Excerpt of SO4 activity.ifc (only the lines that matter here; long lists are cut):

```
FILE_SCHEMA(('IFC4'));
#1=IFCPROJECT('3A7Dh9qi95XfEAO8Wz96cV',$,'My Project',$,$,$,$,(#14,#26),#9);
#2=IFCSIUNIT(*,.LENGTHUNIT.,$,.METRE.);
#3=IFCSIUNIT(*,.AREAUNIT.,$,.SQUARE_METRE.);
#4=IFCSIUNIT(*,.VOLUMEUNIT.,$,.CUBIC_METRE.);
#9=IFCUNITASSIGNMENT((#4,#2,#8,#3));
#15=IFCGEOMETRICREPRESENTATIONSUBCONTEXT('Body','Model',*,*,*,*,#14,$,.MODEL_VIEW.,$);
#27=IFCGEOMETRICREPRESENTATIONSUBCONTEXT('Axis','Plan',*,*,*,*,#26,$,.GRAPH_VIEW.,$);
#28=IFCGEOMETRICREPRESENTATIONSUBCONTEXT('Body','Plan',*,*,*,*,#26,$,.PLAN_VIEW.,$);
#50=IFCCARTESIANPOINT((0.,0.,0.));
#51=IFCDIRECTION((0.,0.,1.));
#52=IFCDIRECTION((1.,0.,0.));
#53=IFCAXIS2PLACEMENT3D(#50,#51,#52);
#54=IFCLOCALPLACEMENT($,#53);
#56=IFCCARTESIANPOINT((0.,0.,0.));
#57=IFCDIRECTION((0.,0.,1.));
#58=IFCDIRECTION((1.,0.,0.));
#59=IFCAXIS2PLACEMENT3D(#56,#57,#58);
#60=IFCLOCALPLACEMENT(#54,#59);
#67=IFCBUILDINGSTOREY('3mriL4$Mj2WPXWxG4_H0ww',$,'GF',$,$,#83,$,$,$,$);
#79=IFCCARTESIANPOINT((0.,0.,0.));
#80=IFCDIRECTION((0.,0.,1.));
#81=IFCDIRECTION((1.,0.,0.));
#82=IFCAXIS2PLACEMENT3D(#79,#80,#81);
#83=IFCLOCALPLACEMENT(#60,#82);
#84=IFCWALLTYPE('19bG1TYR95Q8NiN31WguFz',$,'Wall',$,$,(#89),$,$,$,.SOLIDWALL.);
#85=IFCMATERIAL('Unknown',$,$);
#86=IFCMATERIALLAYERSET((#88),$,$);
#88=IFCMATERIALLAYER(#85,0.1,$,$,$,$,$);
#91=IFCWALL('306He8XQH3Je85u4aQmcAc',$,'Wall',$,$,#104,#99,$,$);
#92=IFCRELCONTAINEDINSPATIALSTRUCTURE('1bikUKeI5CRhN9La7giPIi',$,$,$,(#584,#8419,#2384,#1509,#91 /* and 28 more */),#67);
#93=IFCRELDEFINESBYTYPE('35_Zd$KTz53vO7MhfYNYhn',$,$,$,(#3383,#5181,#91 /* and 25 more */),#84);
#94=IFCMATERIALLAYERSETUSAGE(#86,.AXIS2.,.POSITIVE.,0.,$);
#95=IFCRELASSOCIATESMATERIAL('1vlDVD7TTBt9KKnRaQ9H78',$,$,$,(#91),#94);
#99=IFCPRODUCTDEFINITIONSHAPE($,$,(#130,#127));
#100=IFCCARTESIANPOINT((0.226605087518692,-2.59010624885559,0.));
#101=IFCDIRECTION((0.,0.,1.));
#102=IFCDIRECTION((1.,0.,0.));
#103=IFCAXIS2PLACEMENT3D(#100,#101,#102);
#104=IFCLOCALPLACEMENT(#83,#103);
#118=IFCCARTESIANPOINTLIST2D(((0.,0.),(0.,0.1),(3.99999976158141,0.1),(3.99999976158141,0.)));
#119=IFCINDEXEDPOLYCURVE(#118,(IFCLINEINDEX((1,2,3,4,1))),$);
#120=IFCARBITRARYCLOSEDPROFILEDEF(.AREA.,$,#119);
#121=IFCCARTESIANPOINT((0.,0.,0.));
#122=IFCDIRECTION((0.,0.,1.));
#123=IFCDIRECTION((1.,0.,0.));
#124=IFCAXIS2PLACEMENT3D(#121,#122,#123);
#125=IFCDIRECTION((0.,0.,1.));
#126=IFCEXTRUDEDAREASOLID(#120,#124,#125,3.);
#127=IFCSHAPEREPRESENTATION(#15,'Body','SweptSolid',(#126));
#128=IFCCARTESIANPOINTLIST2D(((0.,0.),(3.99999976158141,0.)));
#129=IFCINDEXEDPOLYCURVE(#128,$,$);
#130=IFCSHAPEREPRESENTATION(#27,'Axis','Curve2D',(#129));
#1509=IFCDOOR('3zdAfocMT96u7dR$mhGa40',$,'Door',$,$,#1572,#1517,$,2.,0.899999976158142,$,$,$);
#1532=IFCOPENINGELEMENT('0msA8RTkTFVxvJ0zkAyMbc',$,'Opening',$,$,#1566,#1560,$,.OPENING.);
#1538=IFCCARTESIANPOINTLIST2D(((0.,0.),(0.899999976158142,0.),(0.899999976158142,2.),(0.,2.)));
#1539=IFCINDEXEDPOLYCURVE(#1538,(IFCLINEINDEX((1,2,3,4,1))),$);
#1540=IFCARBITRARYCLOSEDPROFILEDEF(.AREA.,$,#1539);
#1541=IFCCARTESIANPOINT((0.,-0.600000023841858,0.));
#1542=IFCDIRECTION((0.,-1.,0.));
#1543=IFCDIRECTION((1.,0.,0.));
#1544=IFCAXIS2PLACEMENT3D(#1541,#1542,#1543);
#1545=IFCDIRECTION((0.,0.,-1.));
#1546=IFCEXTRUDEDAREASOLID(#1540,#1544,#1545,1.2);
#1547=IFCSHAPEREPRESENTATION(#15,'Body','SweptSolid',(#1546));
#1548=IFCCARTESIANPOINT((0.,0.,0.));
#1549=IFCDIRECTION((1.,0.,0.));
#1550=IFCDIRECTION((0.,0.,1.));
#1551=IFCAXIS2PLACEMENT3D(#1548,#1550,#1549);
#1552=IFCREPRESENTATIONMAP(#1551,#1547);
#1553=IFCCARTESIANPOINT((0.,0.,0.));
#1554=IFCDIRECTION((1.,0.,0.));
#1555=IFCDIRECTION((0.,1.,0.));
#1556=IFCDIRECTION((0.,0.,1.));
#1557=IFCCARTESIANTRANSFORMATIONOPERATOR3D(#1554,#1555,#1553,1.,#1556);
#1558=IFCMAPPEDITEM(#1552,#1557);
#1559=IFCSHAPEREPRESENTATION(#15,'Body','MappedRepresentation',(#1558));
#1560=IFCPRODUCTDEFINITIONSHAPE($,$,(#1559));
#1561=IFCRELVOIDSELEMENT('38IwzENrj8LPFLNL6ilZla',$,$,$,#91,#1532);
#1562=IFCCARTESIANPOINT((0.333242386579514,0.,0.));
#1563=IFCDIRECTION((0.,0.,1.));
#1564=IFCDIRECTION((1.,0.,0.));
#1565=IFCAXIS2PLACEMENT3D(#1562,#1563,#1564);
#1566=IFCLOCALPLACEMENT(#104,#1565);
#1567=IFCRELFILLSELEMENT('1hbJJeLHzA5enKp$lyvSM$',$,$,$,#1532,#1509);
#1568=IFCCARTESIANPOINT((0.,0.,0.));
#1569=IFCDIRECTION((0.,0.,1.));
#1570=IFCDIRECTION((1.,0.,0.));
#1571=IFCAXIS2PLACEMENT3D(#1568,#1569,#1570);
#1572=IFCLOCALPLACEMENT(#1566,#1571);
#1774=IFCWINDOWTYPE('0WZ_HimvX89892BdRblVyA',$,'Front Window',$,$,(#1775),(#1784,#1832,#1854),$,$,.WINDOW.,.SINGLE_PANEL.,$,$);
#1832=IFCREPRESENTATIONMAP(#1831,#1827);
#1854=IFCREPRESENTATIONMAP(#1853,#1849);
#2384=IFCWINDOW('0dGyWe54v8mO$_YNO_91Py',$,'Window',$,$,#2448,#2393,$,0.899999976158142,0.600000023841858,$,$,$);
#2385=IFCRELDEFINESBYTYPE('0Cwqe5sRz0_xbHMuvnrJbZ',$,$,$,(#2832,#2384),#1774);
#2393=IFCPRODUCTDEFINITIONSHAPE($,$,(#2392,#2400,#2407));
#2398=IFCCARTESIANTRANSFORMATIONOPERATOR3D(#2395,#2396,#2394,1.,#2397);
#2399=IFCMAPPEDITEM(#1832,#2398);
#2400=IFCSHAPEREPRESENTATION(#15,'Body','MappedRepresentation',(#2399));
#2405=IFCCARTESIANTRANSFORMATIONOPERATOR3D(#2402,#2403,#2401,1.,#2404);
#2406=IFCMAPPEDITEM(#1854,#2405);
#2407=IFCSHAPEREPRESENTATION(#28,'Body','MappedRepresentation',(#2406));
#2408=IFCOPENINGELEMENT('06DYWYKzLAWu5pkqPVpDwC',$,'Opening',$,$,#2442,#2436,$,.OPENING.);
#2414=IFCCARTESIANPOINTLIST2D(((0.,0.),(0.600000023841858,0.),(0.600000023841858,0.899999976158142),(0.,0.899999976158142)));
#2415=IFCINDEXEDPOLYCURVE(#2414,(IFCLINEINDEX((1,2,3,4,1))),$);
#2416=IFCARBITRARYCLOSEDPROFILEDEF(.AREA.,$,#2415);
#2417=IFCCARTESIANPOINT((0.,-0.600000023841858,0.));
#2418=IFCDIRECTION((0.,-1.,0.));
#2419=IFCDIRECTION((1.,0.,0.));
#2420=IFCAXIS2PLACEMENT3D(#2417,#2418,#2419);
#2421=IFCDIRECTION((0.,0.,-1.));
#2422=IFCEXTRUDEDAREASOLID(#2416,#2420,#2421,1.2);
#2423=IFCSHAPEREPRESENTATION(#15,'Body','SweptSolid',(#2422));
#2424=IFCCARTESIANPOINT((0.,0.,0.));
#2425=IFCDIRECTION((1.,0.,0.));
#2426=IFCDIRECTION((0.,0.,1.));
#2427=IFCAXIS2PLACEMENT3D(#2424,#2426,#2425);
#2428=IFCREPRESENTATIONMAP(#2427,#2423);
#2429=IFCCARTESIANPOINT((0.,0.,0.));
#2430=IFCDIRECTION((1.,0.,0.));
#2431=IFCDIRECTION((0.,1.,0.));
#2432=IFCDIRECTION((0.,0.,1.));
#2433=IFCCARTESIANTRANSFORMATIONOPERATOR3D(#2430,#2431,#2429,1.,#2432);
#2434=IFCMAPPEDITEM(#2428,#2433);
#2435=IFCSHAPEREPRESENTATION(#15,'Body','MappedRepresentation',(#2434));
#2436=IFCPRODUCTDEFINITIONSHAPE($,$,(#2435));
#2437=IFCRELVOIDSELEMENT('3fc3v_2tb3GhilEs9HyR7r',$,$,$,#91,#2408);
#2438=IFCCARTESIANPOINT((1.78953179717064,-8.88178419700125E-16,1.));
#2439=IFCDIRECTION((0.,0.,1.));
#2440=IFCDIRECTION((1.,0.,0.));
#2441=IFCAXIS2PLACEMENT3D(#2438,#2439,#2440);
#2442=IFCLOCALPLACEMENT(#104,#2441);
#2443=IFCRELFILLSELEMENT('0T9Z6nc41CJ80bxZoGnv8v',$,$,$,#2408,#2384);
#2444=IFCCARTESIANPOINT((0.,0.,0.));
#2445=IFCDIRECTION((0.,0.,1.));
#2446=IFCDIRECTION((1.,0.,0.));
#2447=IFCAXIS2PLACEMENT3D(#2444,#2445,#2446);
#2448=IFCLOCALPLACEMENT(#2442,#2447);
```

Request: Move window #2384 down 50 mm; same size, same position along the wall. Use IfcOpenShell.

```python
import numpy as np
import ifcopenshell
import ifcopenshell.api.geometry
import ifcopenshell.util.placement
import ifcopenshell.util.unit

model = ifcopenshell.open("SO4 activity.ifc")
unit_scale = ifcopenshell.util.unit.calculate_unit_scale(model)

window = model.by_guid("0dGyWe54v8mO$_YNO_91Py")
opening = window.FillsVoids[0].RelatingOpeningElement
dz = -0.05 / unit_scale

shift = np.array([0.0, 0.0, dz])
# The window is placed relative to its opening, so it follows when the opening moves.
matrix = ifcopenshell.util.placement.get_local_placement(opening.ObjectPlacement)
matrix[:3, 3] += shift
ifcopenshell.api.geometry.edit_object_placement(
    model, product=opening, matrix=matrix, is_si=False, should_transform_children=True
)

print(f"moved by {dz * unit_scale:+.3f} m")

model.write("SO4 activity-out.ifc")
```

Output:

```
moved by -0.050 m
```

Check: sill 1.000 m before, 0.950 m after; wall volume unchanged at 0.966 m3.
